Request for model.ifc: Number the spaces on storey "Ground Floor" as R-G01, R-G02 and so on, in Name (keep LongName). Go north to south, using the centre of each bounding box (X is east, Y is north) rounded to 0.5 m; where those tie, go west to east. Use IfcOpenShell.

First a look at what the model holds.

```python
import ifcopenshell
import ifcopenshell.util.element
import ifcopenshell.util.placement

model = ifcopenshell.open("model.ifc")
print(model.schema)
storey = next(s for s in model.by_type("IfcBuildingStorey") if s.Name == "Ground Floor")
spaces = [e for e in ifcopenshell.util.element.get_decomposition(storey) if e.is_a("IfcSpace")]
for e in sorted(spaces, key=lambda e: e.id()):
    origin = ifcopenshell.util.placement.get_local_placement(e.ObjectPlacement)[:3, 3]
    print(e.id(), e.Name, e.LongName, origin.round(2) + 0.0, sep=" | ")
```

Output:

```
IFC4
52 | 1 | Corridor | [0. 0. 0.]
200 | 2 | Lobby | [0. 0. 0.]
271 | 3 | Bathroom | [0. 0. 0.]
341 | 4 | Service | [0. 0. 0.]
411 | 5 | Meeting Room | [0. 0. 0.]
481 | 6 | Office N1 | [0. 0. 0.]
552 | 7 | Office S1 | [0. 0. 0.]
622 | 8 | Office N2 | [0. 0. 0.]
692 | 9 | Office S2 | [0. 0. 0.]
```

```python
import ifcopenshell
import ifcopenshell.geom
import ifcopenshell.util.element
import ifcopenshell.util.shape

model = ifcopenshell.open("model.ifc")
settings = ifcopenshell.geom.settings()
settings.set("use-world-coords", True)


def centre(element):
    shape = ifcopenshell.geom.create_shape(settings, element)
    return ifcopenshell.util.shape.get_bbox_centroid(shape.geometry)


storey = next(s for s in model.by_type("IfcBuildingStorey") if s.Name == "Ground Floor")
spaces = [e for e in ifcopenshell.util.element.get_decomposition(storey) if e.is_a("IfcSpace")]

# Insertion points can sit at a corner or the storey origin, so sort by the geometry (in metres).
centres = {e: centre(e) for e in spaces}
spaces.sort(key=lambda e: (-round(centres[e][1] / 0.5), centres[e][0]))

for i, e in enumerate(spaces, start=1):
    number = f"R-G{i:02d}"
    e.Name = number
    print(e.id(), number)

model.write("model_updated.ifc")
```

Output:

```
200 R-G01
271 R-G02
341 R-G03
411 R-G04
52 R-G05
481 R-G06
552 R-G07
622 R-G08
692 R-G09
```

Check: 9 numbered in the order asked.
